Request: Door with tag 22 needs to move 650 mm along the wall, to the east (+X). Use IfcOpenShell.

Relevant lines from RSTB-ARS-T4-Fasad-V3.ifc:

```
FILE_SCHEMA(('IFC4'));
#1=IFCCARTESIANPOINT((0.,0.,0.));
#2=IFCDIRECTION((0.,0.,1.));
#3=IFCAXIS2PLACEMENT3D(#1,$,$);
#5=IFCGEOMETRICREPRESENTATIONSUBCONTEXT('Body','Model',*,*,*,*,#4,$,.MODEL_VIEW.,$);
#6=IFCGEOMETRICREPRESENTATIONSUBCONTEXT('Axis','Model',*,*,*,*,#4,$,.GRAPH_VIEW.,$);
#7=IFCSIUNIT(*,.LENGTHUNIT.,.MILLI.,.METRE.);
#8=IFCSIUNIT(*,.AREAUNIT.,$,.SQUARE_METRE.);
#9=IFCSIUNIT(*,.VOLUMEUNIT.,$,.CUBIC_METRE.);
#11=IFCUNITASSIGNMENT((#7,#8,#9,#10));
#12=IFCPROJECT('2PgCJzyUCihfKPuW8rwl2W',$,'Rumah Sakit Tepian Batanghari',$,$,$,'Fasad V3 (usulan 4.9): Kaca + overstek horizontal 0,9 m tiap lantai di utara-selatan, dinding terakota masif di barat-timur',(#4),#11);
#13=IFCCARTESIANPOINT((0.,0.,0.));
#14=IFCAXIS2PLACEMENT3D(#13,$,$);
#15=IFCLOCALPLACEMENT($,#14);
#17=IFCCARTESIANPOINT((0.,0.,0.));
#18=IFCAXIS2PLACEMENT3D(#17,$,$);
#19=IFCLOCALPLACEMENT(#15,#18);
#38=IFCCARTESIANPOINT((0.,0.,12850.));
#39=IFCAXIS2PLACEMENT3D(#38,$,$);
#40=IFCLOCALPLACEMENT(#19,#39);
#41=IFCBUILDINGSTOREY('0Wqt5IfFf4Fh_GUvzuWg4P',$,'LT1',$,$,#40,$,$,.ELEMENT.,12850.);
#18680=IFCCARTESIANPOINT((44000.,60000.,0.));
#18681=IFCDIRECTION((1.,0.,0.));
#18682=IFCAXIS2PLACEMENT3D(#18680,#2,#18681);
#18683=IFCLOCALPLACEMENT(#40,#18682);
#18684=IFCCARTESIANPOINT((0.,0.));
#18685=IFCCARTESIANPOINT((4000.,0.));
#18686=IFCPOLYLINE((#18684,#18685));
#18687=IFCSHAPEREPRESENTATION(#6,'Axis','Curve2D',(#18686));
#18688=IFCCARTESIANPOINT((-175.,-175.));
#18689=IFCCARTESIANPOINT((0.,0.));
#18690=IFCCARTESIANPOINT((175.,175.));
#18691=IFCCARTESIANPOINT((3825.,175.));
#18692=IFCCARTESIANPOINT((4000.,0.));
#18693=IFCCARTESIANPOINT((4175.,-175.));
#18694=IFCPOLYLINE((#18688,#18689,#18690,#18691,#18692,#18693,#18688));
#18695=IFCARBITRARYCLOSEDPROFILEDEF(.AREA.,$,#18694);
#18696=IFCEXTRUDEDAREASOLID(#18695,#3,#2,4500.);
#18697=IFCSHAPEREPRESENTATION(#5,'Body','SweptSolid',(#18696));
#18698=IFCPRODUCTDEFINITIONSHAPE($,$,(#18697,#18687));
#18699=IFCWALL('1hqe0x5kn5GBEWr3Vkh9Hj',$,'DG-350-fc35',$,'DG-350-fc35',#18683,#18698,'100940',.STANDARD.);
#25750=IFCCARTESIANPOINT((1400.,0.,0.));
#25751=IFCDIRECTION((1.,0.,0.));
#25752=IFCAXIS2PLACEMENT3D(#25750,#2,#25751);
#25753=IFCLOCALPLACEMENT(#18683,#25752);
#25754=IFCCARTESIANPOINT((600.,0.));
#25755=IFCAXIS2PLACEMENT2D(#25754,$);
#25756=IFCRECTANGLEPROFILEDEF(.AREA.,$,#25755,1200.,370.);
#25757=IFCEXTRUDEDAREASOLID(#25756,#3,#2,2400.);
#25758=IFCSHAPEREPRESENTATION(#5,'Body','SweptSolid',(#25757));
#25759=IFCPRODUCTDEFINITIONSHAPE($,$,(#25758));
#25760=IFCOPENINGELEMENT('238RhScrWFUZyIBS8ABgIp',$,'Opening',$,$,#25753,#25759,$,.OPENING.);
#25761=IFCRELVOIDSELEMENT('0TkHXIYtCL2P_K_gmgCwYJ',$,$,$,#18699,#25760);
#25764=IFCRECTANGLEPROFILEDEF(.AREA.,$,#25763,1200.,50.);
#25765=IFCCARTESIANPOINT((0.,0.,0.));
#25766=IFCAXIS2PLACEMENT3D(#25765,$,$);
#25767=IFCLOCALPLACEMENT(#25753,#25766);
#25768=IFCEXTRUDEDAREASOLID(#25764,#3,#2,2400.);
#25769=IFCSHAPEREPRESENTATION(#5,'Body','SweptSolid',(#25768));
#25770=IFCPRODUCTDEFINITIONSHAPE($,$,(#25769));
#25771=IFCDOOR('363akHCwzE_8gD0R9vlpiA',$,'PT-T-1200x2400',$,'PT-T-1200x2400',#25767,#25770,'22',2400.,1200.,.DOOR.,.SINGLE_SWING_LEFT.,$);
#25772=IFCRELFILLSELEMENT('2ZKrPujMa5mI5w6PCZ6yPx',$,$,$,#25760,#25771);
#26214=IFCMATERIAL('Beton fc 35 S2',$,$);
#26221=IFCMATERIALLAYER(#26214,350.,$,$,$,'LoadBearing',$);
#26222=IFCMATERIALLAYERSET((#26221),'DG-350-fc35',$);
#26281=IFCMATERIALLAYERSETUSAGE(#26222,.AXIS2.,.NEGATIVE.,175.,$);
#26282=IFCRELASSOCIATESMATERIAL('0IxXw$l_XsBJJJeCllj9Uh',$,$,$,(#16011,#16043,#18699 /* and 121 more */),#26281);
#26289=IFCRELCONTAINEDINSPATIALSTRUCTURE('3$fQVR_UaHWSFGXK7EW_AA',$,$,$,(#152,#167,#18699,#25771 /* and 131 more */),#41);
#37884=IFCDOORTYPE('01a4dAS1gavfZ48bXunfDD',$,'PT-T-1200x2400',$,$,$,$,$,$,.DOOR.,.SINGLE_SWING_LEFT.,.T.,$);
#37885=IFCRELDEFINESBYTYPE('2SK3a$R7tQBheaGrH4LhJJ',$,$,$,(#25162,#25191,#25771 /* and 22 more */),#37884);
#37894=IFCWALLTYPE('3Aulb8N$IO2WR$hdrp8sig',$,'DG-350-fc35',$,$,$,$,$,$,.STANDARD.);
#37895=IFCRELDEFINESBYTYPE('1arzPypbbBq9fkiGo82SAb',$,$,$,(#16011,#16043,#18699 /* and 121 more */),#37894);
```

```python
import ifcopenshell
import ifcopenshell.api.geometry
import ifcopenshell.util.placement
import ifcopenshell.util.unit

model = ifcopenshell.open("RSTB-ARS-T4-Fasad-V3.ifc")
unit_scale = ifcopenshell.util.unit.calculate_unit_scale(model)

door = model.by_guid("363akHCwzE_8gD0R9vlpiA")
opening = door.FillsVoids[0].RelatingOpeningElement
wall = opening.VoidsElements[0].RelatingBuildingElement

wall_matrix = ifcopenshell.util.placement.get_local_placement(wall.ObjectPlacement)
shift = wall_matrix[:3, 0] * 0.65 / unit_scale
before = ifcopenshell.util.placement.get_local_placement(door.ObjectPlacement)[:3, 3].copy()

# The door is placed relative to its opening, so it follows when the opening moves.
matrix = ifcopenshell.util.placement.get_local_placement(opening.ObjectPlacement)
matrix[:3, 3] += shift
ifcopenshell.api.geometry.edit_object_placement(
    model, product=opening, matrix=matrix, is_si=False, should_transform_children=True
)

after = ifcopenshell.util.placement.get_local_placement(door.ObjectPlacement)[:3, 3]
print("door moved by", (after - before).round(3) + 0.0)

model.write("RSTB-ARS-T4-Fasad-V3_v2.ifc")
```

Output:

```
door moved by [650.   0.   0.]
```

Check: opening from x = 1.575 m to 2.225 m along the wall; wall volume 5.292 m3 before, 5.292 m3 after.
